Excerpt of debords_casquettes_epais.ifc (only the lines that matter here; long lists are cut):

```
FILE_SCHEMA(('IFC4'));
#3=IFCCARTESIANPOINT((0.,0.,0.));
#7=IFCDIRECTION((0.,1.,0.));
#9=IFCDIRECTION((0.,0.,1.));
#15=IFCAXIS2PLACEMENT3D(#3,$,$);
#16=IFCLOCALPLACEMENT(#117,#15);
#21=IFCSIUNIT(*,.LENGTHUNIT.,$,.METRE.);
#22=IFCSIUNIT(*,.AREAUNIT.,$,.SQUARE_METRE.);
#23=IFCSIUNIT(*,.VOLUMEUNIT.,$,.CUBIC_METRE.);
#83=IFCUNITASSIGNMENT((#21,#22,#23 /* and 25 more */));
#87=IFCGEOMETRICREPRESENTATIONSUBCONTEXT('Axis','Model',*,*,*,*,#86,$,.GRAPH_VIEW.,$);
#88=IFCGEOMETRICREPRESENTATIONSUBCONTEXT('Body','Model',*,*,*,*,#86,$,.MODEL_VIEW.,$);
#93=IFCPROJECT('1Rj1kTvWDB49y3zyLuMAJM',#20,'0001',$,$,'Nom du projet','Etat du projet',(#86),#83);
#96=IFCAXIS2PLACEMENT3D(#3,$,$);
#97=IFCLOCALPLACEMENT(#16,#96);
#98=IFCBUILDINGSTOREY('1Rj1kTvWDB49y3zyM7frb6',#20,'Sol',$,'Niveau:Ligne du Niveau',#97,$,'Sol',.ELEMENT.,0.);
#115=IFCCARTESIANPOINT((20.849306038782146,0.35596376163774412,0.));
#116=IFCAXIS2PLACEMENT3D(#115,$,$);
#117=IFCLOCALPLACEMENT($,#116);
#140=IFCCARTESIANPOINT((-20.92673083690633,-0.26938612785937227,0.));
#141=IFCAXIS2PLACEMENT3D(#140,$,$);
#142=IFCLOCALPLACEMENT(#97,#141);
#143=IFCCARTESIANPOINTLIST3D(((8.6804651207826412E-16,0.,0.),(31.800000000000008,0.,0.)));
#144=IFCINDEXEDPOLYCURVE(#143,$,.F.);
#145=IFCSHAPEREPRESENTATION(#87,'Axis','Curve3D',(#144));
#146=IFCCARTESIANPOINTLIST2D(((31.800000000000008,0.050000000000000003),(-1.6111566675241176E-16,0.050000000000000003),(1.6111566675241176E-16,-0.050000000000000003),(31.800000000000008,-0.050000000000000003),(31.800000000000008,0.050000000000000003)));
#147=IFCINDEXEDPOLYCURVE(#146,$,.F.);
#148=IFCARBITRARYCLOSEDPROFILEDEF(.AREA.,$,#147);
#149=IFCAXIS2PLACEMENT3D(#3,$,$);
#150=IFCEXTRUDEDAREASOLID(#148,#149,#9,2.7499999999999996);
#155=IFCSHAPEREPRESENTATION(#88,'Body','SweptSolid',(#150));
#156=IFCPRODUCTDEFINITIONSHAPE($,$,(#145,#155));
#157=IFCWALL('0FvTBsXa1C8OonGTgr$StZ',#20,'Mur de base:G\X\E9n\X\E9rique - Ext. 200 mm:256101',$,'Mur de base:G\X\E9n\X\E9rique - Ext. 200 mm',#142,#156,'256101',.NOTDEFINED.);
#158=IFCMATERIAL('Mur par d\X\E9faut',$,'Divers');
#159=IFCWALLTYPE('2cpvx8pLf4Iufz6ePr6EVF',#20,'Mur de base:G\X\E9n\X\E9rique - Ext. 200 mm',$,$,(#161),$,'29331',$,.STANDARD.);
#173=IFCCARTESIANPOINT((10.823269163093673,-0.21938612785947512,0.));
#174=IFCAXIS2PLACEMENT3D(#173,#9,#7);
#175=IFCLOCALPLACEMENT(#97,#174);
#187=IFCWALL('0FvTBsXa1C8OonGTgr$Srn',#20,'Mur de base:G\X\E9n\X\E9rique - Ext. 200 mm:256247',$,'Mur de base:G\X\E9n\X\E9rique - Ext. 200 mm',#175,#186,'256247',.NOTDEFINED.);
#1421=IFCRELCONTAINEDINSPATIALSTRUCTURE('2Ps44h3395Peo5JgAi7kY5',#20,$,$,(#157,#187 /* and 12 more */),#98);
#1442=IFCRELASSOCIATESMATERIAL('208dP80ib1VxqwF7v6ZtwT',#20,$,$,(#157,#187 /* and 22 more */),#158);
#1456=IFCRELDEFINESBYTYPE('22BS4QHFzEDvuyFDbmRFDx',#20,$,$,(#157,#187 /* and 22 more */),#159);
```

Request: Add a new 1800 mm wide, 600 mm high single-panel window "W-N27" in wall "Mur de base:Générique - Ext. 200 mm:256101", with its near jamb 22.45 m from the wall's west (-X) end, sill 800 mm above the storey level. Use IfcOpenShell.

```python
import numpy as np
import ifcopenshell
import ifcopenshell.api.feature
import ifcopenshell.api.geometry
import ifcopenshell.api.root
import ifcopenshell.api.spatial
import ifcopenshell.geom
import ifcopenshell.util.element
import ifcopenshell.util.placement
import ifcopenshell.util.representation
import ifcopenshell.util.shape
import ifcopenshell.util.unit

model = ifcopenshell.open("debords_casquettes_epais.ifc")
unit_scale = ifcopenshell.util.unit.calculate_unit_scale(model)
settings = ifcopenshell.geom.settings()


def volume(element):
    """Net volume in cubic metres, openings subtracted."""
    shape = ifcopenshell.geom.create_shape(settings, element)
    return ifcopenshell.util.shape.get_volume(shape.geometry)


wall = model.by_id(157)
storey = ifcopenshell.util.element.get_container(wall, ifc_class="IfcBuildingStorey")
context = ifcopenshell.util.representation.get_context(model, "Model", "Body", "MODEL_VIEW")
before = volume(wall)

width, height, from_end, sill = 1.8, 0.6, 22.45, 0.8  # metres

# The wall runs along its own X axis, and the end named is its -X end.
wall_shape = ifcopenshell.geom.create_shape(settings, wall)
x, y, z = ifcopenshell.util.shape.get_vertices(wall_shape.geometry).T
start = x.min() + from_end
face, thickness = float(y.min()), float(y.max() - y.min())
wall_matrix = ifcopenshell.util.placement.get_local_placement(wall.ObjectPlacement)
level = ifcopenshell.util.placement.get_local_placement(storey.ObjectPlacement)[2, 3]


def in_wall(x, y):
    """Placement at x, y metres in the wall's axes, at sill height."""
    matrix = wall_matrix.copy()
    matrix[:, 3] = wall_matrix @ np.array([x / unit_scale, y / unit_scale, 0.0, 1.0])
    matrix[2, 3] = level + sill / unit_scale
    return matrix


# Opening: a box that overshoots both wall faces by 50 mm.
opening = ifcopenshell.api.root.create_entity(model, ifc_class="IfcOpeningElement", predefined_type="OPENING")
box = ifcopenshell.api.geometry.add_wall_representation(
    model, context=context, length=width, height=height, thickness=thickness + 0.1
)
ifcopenshell.api.geometry.assign_representation(model, product=opening, representation=box)
ifcopenshell.api.geometry.edit_object_placement(model, product=opening, matrix=in_wall(start, face - 0.05), is_si=False)
ifcopenshell.api.feature.add_feature(model, feature=opening, element=wall)

window = ifcopenshell.api.root.create_entity(model, ifc_class="IfcWindow", name="W-N27", predefined_type="WINDOW")
window.OverallWidth, window.OverallHeight = width / unit_scale, height / unit_scale
window.PartitioningType = "SINGLE_PANEL"
body = ifcopenshell.api.geometry.add_window_representation(
    model,
    context=context,
    overall_width=window.OverallWidth,
    overall_height=window.OverallHeight,
    partition_type="SINGLE_PANEL",
)
ifcopenshell.api.geometry.assign_representation(model, product=window, representation=body)
ifcopenshell.api.spatial.assign_container(model, products=[window], relating_structure=storey)
ifcopenshell.api.feature.add_filling(model, opening=opening, element=window)

# Centre the window in the wall's thickness.
ifcopenshell.api.geometry.edit_object_placement(model, product=window, matrix=in_wall(start, face), is_si=False)
window_shape = ifcopenshell.geom.create_shape(settings, window)
depth = ifcopenshell.util.shape.get_vertices(window_shape.geometry)[:, 1]
offset = face + thickness / 2 - (depth.min() + depth.max()) / 2
ifcopenshell.api.geometry.edit_object_placement(model, product=window, matrix=in_wall(start, offset), is_si=False)

after = volume(wall)

print(f"wall volume {before:.3f} -> {after:.3f} m3")

model.write("debords_casquettes_epais_v2.ifc")
```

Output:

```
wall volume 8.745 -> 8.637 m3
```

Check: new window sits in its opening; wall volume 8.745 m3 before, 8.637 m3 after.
